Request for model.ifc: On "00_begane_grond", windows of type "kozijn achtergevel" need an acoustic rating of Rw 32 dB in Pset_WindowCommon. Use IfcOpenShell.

First a look at what the model holds.

```python
import ifcopenshell
import ifcopenshell.util.element

model = ifcopenshell.open("model.ifc")
print(model.schema)
storey = next(s for s in model.by_type("IfcBuildingStorey") if s.Name == "00_begane_grond")
windows = [e for e in ifcopenshell.util.element.get_decomposition(storey) if e.is_a("IfcWindow")]
seen = {}
for e in windows:
    element_type = ifcopenshell.util.element.get_type(e)
    key = (element_type.Name if element_type != e and element_type else None, ifcopenshell.util.element.get_pset(e, "Pset_WindowCommon", "AcousticRating"))
    seen[key] = seen.get(key, 0) + 1
for (name, value), count in sorted(seen.items(), key=str):
    print(count, "x", name, "|", value)
```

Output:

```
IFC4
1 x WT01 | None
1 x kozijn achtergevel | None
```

```python
import ifcopenshell
import ifcopenshell.api.pset
import ifcopenshell.util.element

model = ifcopenshell.open("model.ifc")

storey = next(s for s in model.by_type("IfcBuildingStorey") if s.Name == "00_begane_grond")
windows = [e for e in ifcopenshell.util.element.get_decomposition(storey) if e.is_a("IfcWindow")]

count = 0
for e in windows:
    element_type = ifcopenshell.util.element.get_type(e)
    if element_type in (None, e) or element_type.Name != "kozijn achtergevel":
        continue
    # add_pset returns the element's existing set when there is one.
    pset = ifcopenshell.api.pset.add_pset(model, product=e, name="Pset_WindowCommon")
    ifcopenshell.api.pset.edit_pset(model, pset=pset, properties={"AcousticRating": "Rw 32 dB"})
    count += 1

print(count, "windows updated")

model.write("model-out.ifc")
```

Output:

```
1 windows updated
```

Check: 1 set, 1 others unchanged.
